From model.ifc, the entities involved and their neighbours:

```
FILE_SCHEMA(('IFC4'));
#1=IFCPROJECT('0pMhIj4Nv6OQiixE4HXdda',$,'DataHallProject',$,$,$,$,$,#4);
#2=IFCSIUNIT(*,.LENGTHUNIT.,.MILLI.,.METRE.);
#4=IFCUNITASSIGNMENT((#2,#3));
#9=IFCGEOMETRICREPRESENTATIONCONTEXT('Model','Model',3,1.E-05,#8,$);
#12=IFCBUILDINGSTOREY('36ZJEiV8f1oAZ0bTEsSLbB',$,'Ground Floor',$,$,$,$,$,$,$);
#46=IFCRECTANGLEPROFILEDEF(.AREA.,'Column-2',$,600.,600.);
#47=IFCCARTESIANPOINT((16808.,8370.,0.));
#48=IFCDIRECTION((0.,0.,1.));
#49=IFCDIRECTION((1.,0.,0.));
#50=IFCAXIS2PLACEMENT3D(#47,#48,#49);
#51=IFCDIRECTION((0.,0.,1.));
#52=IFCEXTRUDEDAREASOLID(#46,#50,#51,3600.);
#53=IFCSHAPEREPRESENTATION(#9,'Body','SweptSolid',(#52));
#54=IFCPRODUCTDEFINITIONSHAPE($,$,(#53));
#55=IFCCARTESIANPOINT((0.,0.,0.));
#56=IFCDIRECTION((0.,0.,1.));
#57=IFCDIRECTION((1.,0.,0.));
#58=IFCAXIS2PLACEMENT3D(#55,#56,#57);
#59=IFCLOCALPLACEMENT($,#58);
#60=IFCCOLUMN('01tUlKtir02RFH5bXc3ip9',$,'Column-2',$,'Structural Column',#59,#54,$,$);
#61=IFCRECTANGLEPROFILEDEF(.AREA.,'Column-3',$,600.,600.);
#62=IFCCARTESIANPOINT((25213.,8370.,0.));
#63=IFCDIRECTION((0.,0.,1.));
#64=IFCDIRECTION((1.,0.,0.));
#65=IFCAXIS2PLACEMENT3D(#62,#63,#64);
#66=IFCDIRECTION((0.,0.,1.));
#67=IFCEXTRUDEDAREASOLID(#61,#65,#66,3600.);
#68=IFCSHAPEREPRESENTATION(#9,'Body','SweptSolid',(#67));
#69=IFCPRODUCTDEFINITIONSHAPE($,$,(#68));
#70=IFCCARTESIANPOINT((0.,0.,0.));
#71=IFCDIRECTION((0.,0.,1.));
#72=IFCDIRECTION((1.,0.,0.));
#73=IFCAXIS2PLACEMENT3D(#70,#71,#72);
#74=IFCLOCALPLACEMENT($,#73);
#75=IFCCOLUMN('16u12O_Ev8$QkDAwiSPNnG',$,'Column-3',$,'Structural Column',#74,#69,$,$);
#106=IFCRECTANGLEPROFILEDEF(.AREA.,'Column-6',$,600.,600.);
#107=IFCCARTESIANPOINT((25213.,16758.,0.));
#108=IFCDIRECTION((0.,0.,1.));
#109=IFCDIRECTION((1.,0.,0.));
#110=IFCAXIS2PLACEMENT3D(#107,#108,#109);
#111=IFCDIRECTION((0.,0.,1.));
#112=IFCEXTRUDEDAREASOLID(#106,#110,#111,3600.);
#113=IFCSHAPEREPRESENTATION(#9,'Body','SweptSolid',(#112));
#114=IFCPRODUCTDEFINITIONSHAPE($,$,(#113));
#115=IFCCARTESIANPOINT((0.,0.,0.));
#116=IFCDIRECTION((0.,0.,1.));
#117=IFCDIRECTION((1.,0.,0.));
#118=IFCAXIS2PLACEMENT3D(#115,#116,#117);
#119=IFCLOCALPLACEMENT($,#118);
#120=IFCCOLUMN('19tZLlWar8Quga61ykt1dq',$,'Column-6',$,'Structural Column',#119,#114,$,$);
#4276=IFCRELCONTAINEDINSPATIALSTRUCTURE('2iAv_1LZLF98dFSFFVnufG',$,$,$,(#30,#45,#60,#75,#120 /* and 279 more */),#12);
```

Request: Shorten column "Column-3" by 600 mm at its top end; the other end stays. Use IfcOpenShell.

```python
import ifcopenshell
import ifcopenshell.util.unit

model = ifcopenshell.open("model.ifc")
unit_scale = ifcopenshell.util.unit.calculate_unit_scale(model)

member = model.by_guid("16u12O_Ev8$QkDAwiSPNnG")
change = -0.6 / unit_scale

# The extrusion runs towards the end named, so only its depth changes.
body = next(r for r in member.Representation.Representations if r.RepresentationIdentifier == "Body")
solid = body.Items[0]
old_length = solid.Depth
solid.Depth += change

print(f"length {old_length:g} -> {solid.Depth:g}")

model.write("model_rev.ifc")
```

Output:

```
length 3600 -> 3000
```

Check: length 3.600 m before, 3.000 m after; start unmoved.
